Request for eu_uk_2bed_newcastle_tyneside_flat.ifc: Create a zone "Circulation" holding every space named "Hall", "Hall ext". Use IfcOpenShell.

First a look at what the model holds.

```python
import ifcopenshell

model = ifcopenshell.open("eu_uk_2bed_newcastle_tyneside_flat.ifc")
print(model.schema)
seen = {}
for space in model.by_type("IfcSpace"):
    seen[space.LongName] = seen.get(space.LongName, 0) + 1
for name, count in sorted(seen.items(), key=str):
    print(count, "x", name)
print("zones:", [z.Name for z in model.by_type("IfcZone")][:20])
```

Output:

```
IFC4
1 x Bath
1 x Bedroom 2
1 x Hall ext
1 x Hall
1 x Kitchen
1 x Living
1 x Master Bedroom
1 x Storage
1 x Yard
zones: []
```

```python
import ifcopenshell
import ifcopenshell.api.group
import ifcopenshell.api.root

model = ifcopenshell.open("eu_uk_2bed_newcastle_tyneside_flat.ifc")

names = {"Hall", "Hall ext"}
spaces = [s for s in model.by_type("IfcSpace") if s.LongName in names]

zone = ifcopenshell.api.root.create_entity(model, ifc_class="IfcZone", name="Circulation")
ifcopenshell.api.group.assign_group(model, products=spaces, group=zone)
print(len(spaces), "spaces in", zone.Name)

model.write("eu_uk_2bed_newcastle_tyneside_flat_updated.ifc")
```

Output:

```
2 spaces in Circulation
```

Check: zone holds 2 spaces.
